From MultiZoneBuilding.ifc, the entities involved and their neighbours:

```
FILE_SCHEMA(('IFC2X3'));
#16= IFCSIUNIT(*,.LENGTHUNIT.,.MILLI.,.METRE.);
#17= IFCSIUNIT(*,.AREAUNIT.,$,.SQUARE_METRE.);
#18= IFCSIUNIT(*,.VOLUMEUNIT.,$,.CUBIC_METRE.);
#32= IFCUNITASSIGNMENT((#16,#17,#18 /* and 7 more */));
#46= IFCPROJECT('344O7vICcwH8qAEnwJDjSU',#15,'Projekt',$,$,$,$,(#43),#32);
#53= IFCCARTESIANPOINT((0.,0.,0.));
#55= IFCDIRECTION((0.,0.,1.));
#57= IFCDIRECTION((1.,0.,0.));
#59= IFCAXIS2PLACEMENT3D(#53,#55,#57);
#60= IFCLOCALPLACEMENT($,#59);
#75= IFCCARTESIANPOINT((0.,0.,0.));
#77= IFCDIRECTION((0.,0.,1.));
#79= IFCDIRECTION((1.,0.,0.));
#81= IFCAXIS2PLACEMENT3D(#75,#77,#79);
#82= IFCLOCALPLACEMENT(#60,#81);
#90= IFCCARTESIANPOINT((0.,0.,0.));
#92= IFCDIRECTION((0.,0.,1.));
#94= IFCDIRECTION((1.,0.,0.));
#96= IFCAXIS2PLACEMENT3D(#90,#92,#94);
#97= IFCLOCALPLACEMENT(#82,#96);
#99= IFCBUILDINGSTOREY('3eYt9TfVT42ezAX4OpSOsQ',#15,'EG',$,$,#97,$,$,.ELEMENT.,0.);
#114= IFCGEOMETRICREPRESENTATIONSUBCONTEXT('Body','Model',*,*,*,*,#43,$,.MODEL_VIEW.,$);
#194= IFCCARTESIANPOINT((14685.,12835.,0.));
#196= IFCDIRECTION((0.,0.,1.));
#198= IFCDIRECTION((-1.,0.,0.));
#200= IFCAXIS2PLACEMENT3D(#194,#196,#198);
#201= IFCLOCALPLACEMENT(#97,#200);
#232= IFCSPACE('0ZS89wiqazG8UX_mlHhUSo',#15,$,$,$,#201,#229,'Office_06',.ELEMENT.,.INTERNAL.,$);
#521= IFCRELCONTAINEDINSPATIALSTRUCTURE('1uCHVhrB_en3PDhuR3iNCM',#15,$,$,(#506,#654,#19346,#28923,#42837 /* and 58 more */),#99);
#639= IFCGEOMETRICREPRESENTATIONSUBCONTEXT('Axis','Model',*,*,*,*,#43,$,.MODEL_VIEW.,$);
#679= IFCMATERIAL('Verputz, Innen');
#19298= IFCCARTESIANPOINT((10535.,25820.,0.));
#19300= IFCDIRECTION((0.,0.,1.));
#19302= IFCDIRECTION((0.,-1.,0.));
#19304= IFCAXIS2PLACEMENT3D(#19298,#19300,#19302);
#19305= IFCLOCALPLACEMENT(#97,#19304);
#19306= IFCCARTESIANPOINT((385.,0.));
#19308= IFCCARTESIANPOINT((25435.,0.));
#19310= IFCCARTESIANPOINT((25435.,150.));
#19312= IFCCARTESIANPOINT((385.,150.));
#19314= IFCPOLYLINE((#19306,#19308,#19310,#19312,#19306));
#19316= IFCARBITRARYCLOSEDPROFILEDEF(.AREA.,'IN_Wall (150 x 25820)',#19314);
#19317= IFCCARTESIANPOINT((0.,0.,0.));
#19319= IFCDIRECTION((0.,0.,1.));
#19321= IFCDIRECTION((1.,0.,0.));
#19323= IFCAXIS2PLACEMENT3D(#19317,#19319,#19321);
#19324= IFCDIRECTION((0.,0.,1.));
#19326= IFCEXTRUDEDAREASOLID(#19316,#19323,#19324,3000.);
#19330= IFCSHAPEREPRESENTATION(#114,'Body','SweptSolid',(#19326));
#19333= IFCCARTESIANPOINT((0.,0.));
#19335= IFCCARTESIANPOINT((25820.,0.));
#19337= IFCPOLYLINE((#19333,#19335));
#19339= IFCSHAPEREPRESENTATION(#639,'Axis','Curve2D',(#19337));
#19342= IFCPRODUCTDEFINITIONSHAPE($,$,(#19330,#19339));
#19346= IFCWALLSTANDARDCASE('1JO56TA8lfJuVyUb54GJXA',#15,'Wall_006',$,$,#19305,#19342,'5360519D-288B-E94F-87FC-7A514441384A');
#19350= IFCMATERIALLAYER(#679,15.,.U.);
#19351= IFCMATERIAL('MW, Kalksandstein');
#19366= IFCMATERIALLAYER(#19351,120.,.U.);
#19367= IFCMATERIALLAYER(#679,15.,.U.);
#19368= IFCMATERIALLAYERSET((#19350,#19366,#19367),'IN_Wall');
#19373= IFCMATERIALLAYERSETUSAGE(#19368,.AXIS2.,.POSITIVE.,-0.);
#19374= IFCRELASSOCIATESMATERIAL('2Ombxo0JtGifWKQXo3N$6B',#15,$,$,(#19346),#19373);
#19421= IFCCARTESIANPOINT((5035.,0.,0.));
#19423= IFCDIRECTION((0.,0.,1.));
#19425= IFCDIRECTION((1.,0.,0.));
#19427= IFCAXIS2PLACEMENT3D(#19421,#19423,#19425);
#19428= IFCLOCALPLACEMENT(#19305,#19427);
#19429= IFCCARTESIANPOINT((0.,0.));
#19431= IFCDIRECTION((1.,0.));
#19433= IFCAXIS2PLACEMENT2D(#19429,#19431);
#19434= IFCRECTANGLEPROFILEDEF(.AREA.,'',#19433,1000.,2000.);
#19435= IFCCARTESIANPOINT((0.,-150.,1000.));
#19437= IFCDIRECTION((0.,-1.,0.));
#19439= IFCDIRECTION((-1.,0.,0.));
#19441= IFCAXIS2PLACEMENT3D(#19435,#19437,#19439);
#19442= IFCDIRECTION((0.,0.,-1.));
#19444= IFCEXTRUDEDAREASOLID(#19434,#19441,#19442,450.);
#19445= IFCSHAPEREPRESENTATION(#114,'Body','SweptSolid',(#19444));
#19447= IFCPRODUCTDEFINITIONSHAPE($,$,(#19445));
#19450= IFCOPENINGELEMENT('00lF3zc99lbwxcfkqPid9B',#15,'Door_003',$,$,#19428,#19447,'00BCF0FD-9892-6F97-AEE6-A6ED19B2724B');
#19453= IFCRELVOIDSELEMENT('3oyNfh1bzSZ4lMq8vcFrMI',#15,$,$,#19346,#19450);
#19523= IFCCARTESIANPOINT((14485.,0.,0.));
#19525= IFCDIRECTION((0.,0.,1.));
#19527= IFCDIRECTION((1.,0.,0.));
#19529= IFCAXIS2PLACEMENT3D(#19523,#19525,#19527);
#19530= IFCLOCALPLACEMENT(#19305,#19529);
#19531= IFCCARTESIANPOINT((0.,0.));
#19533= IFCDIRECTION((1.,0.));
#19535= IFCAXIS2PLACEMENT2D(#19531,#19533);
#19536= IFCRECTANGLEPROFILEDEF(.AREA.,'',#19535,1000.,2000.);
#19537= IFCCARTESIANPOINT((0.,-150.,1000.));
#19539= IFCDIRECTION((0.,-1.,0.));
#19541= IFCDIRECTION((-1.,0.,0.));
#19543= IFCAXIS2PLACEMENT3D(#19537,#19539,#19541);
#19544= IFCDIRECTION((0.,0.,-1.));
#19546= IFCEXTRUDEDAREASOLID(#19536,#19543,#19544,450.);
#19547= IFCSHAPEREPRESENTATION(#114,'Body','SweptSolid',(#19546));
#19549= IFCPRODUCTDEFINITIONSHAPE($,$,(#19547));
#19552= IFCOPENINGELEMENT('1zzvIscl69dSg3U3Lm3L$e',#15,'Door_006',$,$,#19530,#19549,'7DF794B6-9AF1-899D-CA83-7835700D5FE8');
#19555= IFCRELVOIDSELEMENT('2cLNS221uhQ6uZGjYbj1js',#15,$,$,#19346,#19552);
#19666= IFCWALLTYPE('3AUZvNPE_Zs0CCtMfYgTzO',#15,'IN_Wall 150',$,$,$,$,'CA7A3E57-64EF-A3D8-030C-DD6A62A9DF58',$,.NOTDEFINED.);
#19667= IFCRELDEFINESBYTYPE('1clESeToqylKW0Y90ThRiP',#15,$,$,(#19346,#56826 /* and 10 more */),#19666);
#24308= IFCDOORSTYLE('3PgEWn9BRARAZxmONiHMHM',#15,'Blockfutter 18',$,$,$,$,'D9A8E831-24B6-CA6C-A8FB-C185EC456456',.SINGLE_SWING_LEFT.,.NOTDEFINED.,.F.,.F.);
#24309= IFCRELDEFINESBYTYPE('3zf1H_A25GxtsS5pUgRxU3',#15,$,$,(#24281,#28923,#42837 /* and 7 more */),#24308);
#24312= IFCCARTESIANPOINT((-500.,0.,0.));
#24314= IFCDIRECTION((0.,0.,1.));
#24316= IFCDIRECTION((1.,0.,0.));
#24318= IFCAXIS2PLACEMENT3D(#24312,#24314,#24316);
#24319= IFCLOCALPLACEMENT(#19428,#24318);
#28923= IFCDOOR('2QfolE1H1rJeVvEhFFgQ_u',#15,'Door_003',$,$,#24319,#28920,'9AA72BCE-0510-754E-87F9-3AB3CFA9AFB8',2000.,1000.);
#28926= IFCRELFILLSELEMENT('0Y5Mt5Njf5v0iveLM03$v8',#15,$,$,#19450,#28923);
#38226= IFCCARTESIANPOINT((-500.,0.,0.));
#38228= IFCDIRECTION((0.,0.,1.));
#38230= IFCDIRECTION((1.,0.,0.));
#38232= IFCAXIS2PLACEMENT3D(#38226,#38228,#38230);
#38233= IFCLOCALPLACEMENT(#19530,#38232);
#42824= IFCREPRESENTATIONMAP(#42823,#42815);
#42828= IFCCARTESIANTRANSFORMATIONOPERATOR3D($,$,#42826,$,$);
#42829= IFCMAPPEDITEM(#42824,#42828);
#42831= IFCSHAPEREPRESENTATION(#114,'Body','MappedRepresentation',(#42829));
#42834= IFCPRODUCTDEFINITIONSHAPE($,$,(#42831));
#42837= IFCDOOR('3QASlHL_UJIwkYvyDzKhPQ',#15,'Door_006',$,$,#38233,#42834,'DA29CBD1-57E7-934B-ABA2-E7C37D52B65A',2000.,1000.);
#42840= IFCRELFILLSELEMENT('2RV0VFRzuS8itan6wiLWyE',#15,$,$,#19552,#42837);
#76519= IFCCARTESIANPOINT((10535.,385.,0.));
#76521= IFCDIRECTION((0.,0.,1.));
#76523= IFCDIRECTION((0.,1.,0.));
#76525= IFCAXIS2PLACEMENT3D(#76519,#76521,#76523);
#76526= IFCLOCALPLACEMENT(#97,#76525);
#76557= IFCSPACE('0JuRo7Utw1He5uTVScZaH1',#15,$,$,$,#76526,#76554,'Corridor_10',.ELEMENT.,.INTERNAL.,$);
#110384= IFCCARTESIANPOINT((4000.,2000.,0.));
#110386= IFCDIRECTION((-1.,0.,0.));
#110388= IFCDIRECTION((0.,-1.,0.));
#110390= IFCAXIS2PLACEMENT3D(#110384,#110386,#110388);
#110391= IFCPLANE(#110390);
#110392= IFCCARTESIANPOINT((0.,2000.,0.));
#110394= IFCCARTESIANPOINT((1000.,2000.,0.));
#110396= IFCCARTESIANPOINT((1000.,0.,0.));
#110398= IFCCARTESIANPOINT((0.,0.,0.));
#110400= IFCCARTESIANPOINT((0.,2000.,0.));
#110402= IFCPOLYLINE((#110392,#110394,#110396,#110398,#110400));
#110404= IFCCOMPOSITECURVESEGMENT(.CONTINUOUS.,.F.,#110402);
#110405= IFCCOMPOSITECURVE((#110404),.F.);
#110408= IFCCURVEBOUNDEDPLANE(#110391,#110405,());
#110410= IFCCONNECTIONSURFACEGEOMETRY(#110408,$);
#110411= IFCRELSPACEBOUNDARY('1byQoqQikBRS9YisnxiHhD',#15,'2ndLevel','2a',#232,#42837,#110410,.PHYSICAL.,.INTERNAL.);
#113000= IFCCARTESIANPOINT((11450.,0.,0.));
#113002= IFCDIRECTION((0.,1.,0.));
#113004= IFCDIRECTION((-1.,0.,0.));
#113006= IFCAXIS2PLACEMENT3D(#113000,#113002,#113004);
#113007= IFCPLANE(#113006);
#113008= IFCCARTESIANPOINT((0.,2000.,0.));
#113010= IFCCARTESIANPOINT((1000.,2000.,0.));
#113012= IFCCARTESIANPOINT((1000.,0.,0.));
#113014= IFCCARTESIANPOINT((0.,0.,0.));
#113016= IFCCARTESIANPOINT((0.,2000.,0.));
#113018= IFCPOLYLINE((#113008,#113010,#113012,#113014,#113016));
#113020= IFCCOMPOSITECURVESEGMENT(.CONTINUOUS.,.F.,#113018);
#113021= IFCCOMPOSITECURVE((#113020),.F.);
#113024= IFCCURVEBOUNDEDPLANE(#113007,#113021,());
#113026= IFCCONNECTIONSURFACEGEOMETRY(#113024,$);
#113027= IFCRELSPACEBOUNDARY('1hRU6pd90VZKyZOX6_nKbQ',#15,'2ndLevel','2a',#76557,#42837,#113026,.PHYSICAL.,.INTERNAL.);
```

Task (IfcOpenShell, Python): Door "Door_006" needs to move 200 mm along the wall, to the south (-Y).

```python
import numpy as np
import ifcopenshell
import ifcopenshell.api.geometry
import ifcopenshell.util.placement
import ifcopenshell.util.unit

model = ifcopenshell.open("MultiZoneBuilding.ifc")
unit_scale = ifcopenshell.util.unit.calculate_unit_scale(model)

door = model.by_guid("3QASlHL_UJIwkYvyDzKhPQ")
opening = door.FillsVoids[0].RelatingOpeningElement
wall = opening.VoidsElements[0].RelatingBuildingElement

wall_matrix = ifcopenshell.util.placement.get_local_placement(wall.ObjectPlacement)
shift = wall_matrix[:3, 0] * 0.2 / unit_scale
before = ifcopenshell.util.placement.get_local_placement(door.ObjectPlacement)[:3, 3].copy()

# The door is placed relative to its opening, so it follows when the opening moves.
matrix = ifcopenshell.util.placement.get_local_placement(opening.ObjectPlacement)
matrix[:3, 3] += shift
ifcopenshell.api.geometry.edit_object_placement(
    model, product=opening, matrix=matrix, is_si=False, should_transform_children=True
)

# Space boundary surfaces are stored in each space's coordinates; move them too.
for rel in door.ProvidesBoundaries:
    if not rel.ConnectionGeometry:
        continue
    surface = rel.ConnectionGeometry.SurfaceOnRelatingElement.BasisSurface
    space_matrix = ifcopenshell.util.placement.get_local_placement(rel.RelatingSpace.ObjectPlacement)
    point = np.array(surface.Position.Location.Coordinates) + space_matrix[:3, :3].T @ shift
    surface.Position = model.createIfcAxis2Placement3D(
        model.createIfcCartesianPoint(point.tolist()), surface.Position.Axis, surface.Position.RefDirection
    )

after = ifcopenshell.util.placement.get_local_placement(door.ObjectPlacement)[:3, 3]
print("door moved by", (after - before).round(3) + 0.0)

model.write("MultiZoneBuilding_edited.ifc")
```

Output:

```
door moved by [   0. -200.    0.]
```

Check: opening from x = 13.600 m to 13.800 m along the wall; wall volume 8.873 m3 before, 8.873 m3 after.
